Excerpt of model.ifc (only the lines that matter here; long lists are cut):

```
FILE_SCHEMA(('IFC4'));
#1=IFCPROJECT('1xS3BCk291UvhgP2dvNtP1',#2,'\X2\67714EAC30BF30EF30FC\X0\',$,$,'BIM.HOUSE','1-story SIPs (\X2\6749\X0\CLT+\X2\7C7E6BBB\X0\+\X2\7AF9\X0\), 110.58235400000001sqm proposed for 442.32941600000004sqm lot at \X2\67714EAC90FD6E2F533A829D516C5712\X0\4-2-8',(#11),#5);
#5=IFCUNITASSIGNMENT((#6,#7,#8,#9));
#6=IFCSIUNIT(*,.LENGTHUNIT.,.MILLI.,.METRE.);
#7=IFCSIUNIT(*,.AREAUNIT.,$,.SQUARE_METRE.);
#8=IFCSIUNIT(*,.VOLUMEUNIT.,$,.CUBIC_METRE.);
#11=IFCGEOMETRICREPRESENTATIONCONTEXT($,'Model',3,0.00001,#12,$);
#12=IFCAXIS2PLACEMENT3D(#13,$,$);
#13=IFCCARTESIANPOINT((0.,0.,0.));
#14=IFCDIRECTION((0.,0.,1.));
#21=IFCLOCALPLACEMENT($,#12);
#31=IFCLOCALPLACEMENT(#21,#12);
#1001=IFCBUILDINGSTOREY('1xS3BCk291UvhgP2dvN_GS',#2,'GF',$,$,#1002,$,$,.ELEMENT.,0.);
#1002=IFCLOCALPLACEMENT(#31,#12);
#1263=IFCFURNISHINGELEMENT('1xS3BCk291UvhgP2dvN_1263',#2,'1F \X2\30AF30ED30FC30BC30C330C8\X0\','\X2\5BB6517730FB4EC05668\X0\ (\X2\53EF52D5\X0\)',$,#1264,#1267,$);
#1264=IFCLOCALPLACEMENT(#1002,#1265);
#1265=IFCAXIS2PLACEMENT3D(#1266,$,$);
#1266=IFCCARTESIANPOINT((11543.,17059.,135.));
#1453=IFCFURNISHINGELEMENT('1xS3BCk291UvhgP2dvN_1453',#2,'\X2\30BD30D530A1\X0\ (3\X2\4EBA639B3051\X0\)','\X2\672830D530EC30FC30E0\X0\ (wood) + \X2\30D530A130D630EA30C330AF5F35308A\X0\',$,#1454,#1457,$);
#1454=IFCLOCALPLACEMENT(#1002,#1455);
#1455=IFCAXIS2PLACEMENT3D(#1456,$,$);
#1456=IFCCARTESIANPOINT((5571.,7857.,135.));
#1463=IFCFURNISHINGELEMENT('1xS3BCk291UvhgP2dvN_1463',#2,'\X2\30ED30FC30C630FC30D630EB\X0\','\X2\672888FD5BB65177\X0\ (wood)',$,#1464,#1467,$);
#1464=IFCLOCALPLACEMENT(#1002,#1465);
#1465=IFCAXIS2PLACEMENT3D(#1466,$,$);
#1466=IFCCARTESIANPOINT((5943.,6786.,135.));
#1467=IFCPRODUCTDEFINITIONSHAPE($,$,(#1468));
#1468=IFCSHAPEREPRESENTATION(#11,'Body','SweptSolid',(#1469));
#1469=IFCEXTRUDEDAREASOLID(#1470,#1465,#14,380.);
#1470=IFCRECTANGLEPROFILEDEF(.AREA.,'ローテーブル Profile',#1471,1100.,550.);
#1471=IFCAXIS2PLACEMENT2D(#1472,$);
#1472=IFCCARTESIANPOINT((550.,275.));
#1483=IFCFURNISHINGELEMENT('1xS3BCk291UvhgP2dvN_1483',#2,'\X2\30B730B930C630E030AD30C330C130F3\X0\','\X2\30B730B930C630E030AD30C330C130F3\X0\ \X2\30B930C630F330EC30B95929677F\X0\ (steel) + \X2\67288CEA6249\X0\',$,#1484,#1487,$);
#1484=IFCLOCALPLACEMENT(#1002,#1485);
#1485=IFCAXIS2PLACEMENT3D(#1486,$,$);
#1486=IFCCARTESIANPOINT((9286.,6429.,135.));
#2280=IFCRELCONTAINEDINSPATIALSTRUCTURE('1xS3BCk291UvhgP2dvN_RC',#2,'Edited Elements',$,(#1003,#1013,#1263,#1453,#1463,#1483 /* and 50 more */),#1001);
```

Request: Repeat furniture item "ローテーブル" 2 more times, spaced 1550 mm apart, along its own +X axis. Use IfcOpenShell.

```python
import ifcopenshell
import ifcopenshell.api.geometry
import ifcopenshell.api.root
import ifcopenshell.util.element
import ifcopenshell.util.placement

model = ifcopenshell.open("model.ifc")


def reuse_history(source, copy):
    """copy_class also copies each property set's owner history, people and application; keep the originals."""
    for rel in copy.IsDefinedBy:
        if rel.is_a("IfcRelDefinesByProperties") and (history := rel.RelatingPropertyDefinition.OwnerHistory):
            rel.RelatingPropertyDefinition.OwnerHistory = source.OwnerHistory
            ifcopenshell.util.element.remove_deep2(model, history)


source = model.by_id(1463)
base = ifcopenshell.util.placement.get_local_placement(source.ObjectPlacement)
step = base[:3, 0] * 1550.0

for i in range(1, 3):
    copy = ifcopenshell.api.root.copy_class(model, product=source)
    copy.Representation = ifcopenshell.util.element.copy_deep(
        model, source.Representation, exclude=["IfcGeometricRepresentationContext", "IfcRepresentationMap"]
    )
    reuse_history(source, copy)
    matrix = base.copy()
    matrix[:3, 3] += i * step
    print("added at", matrix[:3, 3].round(3) + 0.0)
    ifcopenshell.api.geometry.edit_object_placement(model, product=copy, matrix=matrix, is_si=False)

model.write("model_rev.ifc")
```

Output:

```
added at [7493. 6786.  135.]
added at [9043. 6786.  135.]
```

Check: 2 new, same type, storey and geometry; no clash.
